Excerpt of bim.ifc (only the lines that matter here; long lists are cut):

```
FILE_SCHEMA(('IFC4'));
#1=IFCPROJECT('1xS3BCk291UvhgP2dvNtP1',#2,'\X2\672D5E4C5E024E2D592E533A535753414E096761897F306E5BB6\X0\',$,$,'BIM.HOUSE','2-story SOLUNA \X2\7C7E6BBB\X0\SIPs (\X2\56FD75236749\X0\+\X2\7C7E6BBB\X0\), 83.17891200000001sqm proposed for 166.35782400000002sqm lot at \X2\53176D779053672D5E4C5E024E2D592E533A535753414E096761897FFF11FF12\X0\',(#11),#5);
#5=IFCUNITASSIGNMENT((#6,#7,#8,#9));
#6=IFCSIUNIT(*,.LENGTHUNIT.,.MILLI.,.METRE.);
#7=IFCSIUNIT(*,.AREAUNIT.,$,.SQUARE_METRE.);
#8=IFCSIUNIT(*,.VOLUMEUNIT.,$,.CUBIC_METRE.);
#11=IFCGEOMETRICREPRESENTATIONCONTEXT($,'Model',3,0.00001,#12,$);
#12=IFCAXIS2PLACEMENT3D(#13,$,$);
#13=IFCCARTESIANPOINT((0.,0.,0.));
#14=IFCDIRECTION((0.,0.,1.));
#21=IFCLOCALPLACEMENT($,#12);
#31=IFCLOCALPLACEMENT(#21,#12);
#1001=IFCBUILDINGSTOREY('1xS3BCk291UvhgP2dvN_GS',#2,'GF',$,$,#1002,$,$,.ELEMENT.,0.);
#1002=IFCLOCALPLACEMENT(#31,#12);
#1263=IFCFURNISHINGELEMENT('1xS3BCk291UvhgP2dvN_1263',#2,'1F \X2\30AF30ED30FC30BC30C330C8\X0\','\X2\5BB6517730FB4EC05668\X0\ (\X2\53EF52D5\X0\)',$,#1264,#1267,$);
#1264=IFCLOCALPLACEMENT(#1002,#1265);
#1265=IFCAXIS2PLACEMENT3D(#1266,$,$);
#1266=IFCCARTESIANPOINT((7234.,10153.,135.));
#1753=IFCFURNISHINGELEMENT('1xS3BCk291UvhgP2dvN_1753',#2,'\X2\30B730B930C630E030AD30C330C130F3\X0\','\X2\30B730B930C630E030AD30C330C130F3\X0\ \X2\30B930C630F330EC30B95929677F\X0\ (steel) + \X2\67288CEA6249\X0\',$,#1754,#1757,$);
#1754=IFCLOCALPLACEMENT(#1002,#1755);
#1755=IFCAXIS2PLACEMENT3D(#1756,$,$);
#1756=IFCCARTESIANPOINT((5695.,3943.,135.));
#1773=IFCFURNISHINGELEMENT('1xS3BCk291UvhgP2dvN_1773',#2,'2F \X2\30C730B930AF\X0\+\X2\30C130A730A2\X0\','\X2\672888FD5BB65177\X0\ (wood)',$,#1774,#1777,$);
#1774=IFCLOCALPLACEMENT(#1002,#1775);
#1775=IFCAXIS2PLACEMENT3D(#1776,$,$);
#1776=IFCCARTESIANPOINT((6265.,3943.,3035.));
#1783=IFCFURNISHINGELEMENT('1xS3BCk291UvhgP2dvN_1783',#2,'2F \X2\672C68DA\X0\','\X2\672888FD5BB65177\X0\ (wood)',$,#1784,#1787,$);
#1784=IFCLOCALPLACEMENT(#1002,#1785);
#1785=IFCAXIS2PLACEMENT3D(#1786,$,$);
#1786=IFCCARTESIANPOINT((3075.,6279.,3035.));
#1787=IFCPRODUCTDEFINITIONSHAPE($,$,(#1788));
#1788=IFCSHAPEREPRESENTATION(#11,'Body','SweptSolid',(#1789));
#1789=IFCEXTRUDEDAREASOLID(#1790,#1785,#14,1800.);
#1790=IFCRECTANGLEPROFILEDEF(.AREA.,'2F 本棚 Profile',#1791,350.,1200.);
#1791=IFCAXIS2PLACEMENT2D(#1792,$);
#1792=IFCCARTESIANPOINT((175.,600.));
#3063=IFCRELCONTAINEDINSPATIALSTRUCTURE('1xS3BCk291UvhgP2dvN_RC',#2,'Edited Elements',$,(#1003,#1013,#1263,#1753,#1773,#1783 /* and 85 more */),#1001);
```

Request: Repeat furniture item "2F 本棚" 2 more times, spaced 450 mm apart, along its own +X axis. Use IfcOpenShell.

```python
import ifcopenshell
import ifcopenshell.api.geometry
import ifcopenshell.api.root
import ifcopenshell.util.element
import ifcopenshell.util.placement

model = ifcopenshell.open("bim.ifc")


def reuse_history(source, copy):
    """copy_class also copies each property set's owner history, people and application; keep the originals."""
    for rel in copy.IsDefinedBy:
        if rel.is_a("IfcRelDefinesByProperties") and (history := rel.RelatingPropertyDefinition.OwnerHistory):
            rel.RelatingPropertyDefinition.OwnerHistory = source.OwnerHistory
            ifcopenshell.util.element.remove_deep2(model, history)


source = model.by_id(1783)
base = ifcopenshell.util.placement.get_local_placement(source.ObjectPlacement)
step = base[:3, 0] * 450.0

for i in range(1, 3):
    copy = ifcopenshell.api.root.copy_class(model, product=source)
    copy.Representation = ifcopenshell.util.element.copy_deep(
        model, source.Representation, exclude=["IfcGeometricRepresentationContext", "IfcRepresentationMap"]
    )
    reuse_history(source, copy)
    matrix = base.copy()
    matrix[:3, 3] += i * step
    print("added at", matrix[:3, 3].round(3) + 0.0)
    ifcopenshell.api.geometry.edit_object_placement(model, product=copy, matrix=matrix, is_si=False)

model.write("bim_edited.ifc")
```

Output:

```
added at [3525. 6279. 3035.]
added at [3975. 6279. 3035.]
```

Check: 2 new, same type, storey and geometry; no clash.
